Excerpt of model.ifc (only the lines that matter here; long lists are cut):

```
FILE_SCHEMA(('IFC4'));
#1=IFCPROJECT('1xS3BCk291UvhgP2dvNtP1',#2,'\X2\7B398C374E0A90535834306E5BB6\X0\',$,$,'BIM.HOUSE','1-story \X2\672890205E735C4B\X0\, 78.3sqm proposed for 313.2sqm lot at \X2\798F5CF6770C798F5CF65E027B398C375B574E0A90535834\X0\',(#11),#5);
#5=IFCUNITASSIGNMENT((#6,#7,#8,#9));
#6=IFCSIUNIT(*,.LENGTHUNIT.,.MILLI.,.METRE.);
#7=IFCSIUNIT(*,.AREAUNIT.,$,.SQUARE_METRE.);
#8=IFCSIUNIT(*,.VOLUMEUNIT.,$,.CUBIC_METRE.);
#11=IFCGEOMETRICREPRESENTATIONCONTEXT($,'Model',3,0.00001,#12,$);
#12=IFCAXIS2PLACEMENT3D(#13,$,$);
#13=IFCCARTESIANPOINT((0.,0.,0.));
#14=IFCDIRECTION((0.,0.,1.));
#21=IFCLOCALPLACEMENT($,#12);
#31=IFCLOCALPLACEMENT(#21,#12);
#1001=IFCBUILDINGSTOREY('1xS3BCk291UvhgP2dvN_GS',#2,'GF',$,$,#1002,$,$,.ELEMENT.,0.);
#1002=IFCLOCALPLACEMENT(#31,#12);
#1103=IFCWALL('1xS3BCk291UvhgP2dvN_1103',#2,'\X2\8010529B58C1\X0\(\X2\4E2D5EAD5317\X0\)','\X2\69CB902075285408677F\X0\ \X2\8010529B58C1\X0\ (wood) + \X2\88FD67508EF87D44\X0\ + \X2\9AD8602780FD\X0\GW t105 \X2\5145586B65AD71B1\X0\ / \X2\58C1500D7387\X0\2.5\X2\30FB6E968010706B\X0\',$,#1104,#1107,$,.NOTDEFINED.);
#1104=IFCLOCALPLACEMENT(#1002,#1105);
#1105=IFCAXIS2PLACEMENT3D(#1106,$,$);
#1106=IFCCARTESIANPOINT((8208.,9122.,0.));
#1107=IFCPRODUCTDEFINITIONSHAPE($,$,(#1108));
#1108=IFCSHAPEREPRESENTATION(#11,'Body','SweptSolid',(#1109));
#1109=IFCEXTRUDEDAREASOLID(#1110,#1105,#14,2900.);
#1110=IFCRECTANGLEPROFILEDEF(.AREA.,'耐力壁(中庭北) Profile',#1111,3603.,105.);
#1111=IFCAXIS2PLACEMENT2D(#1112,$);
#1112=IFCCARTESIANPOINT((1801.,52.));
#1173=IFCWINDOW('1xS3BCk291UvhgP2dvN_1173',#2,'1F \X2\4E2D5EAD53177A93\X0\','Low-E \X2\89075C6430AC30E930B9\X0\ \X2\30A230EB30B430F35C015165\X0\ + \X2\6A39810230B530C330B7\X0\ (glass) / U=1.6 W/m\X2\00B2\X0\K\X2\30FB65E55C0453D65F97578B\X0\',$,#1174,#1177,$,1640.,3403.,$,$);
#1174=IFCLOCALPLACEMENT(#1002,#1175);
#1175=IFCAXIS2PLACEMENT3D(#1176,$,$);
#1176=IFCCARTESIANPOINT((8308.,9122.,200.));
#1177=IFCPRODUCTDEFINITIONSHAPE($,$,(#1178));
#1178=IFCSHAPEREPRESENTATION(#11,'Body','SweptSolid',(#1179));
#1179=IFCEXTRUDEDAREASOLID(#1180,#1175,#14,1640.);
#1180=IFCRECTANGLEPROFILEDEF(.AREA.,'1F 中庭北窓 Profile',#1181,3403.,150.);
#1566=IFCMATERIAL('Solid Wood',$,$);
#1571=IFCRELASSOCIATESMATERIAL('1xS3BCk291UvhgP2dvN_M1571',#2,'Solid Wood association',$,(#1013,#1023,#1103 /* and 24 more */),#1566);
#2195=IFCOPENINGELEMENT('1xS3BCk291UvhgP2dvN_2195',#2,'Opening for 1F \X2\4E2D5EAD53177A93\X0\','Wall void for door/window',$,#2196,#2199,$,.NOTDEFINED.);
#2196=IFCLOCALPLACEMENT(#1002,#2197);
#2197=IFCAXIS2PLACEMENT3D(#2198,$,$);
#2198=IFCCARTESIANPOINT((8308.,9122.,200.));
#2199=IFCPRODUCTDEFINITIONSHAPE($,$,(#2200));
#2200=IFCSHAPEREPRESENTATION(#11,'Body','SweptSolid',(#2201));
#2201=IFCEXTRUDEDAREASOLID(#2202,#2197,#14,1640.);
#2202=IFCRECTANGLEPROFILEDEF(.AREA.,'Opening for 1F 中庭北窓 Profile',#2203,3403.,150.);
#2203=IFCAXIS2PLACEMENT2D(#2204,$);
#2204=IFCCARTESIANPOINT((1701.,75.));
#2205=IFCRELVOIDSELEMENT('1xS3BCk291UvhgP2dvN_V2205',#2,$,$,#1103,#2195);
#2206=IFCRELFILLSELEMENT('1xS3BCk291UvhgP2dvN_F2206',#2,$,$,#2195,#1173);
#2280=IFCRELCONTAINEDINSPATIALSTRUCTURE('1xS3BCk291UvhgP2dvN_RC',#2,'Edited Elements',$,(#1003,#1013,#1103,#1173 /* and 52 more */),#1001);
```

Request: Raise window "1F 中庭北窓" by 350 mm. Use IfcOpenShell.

```python
import numpy as np
import ifcopenshell
import ifcopenshell.api.geometry
import ifcopenshell.util.placement
import ifcopenshell.util.unit

model = ifcopenshell.open("model.ifc")
unit_scale = ifcopenshell.util.unit.calculate_unit_scale(model)

window = model.by_guid("1xS3BCk291UvhgP2dvN_1173")
opening = window.FillsVoids[0].RelatingOpeningElement
dz = 350.0

shift = np.array([0.0, 0.0, dz])
# The window is not placed relative to its opening, so move both.
for product in (opening, window):
    matrix = ifcopenshell.util.placement.get_local_placement(product.ObjectPlacement)
    matrix[:3, 3] += shift
    ifcopenshell.api.geometry.edit_object_placement(model, product=product, matrix=matrix, is_si=False)

print(f"moved by {dz * unit_scale:+.3f} m")

model.write("model_updated.ifc")
```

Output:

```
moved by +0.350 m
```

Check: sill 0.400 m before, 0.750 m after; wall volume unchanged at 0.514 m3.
